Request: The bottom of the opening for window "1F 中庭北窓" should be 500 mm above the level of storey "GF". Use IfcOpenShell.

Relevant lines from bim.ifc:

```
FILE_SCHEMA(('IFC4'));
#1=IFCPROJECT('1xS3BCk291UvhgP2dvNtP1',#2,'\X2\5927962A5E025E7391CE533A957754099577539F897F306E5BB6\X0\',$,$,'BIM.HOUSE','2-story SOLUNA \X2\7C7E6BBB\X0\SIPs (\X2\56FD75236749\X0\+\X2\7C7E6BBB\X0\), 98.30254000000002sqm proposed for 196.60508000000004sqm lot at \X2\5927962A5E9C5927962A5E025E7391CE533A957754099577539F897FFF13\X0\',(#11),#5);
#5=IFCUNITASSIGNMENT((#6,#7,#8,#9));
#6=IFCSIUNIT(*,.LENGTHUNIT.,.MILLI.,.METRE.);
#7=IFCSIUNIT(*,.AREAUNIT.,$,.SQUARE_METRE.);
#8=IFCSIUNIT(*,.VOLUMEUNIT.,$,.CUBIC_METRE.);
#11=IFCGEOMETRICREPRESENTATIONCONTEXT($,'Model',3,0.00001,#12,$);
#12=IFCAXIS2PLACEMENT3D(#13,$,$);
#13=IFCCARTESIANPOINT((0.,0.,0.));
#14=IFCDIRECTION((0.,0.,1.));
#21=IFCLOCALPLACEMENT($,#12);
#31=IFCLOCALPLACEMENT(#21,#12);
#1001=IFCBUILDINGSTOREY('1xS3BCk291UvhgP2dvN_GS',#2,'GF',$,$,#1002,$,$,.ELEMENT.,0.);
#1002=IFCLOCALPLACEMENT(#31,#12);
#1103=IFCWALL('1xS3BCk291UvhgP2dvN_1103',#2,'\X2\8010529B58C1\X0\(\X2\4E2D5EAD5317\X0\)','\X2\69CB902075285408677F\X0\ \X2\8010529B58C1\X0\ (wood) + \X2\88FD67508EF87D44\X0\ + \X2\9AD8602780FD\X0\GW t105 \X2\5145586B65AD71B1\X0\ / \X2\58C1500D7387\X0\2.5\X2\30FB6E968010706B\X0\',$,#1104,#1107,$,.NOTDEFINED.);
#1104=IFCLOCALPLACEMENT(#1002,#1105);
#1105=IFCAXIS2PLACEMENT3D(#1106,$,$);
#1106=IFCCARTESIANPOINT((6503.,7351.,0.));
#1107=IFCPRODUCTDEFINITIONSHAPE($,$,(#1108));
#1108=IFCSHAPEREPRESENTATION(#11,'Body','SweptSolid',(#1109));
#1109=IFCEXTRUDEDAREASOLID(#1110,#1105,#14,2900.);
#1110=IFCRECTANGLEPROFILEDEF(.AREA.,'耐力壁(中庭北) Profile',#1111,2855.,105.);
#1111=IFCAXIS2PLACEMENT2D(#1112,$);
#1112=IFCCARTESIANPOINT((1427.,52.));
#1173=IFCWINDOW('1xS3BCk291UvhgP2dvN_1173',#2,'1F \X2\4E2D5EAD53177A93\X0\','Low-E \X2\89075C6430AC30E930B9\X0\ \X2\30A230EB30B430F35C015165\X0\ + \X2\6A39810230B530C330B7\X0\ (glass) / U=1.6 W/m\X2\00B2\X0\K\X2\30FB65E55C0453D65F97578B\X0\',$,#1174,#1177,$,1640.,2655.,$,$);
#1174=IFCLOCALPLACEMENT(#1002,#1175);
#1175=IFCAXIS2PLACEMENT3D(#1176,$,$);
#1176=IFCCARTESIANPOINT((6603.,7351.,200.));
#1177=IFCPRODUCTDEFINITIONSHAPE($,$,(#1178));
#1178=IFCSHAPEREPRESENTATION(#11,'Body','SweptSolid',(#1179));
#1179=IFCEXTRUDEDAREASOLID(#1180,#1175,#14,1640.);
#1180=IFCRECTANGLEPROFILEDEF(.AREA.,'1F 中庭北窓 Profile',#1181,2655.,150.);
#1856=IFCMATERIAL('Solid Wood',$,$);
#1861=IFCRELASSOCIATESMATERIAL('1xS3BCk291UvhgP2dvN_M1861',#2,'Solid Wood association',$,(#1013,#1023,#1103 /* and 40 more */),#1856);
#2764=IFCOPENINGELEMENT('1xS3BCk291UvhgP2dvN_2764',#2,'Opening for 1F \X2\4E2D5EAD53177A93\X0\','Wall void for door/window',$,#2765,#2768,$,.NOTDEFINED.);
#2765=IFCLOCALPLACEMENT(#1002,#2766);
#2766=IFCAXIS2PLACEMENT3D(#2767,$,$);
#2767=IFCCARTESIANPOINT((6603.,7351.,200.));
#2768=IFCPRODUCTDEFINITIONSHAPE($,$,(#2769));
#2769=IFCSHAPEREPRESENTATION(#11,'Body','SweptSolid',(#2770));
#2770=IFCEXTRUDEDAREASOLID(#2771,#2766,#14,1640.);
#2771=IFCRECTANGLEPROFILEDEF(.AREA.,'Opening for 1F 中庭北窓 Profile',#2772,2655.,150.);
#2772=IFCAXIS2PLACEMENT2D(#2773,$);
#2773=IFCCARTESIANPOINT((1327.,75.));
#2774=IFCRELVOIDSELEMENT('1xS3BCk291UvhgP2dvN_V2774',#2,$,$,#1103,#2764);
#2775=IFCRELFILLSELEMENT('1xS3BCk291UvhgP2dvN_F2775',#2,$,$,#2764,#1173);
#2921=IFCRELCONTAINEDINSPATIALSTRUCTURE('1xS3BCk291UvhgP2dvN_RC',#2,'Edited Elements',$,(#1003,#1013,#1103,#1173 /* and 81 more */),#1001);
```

```python
import numpy as np
import ifcopenshell
import ifcopenshell.api.geometry
import ifcopenshell.geom
import ifcopenshell.util.element
import ifcopenshell.util.placement
import ifcopenshell.util.shape
import ifcopenshell.util.unit

model = ifcopenshell.open("bim.ifc")
unit_scale = ifcopenshell.util.unit.calculate_unit_scale(model)

window = model.by_guid("1xS3BCk291UvhgP2dvN_1173")
opening = window.FillsVoids[0].RelatingOpeningElement
storey = ifcopenshell.util.element.get_container(window, ifc_class="IfcBuildingStorey")
level = ifcopenshell.util.placement.get_local_placement(storey.ObjectPlacement)[2, 3]

# The opening's origin need not be at the sill, so measure its lowest point.
shape = ifcopenshell.geom.create_shape(ifcopenshell.geom.settings(), opening)
bottom = ifcopenshell.util.shape.get_shape_bottom_elevation(shape, shape.geometry) / unit_scale
dz = level + 0.5 / unit_scale - bottom

shift = np.array([0.0, 0.0, dz])
# The window is not placed relative to its opening, so move both.
for product in (opening, window):
    matrix = ifcopenshell.util.placement.get_local_placement(product.ObjectPlacement)
    matrix[:3, 3] += shift
    ifcopenshell.api.geometry.edit_object_placement(model, product=product, matrix=matrix, is_si=False)

print(f"moved by {dz * unit_scale:+.3f} m")

model.write("bim_updated.ifc")
```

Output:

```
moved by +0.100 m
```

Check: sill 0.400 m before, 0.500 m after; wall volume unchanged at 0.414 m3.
